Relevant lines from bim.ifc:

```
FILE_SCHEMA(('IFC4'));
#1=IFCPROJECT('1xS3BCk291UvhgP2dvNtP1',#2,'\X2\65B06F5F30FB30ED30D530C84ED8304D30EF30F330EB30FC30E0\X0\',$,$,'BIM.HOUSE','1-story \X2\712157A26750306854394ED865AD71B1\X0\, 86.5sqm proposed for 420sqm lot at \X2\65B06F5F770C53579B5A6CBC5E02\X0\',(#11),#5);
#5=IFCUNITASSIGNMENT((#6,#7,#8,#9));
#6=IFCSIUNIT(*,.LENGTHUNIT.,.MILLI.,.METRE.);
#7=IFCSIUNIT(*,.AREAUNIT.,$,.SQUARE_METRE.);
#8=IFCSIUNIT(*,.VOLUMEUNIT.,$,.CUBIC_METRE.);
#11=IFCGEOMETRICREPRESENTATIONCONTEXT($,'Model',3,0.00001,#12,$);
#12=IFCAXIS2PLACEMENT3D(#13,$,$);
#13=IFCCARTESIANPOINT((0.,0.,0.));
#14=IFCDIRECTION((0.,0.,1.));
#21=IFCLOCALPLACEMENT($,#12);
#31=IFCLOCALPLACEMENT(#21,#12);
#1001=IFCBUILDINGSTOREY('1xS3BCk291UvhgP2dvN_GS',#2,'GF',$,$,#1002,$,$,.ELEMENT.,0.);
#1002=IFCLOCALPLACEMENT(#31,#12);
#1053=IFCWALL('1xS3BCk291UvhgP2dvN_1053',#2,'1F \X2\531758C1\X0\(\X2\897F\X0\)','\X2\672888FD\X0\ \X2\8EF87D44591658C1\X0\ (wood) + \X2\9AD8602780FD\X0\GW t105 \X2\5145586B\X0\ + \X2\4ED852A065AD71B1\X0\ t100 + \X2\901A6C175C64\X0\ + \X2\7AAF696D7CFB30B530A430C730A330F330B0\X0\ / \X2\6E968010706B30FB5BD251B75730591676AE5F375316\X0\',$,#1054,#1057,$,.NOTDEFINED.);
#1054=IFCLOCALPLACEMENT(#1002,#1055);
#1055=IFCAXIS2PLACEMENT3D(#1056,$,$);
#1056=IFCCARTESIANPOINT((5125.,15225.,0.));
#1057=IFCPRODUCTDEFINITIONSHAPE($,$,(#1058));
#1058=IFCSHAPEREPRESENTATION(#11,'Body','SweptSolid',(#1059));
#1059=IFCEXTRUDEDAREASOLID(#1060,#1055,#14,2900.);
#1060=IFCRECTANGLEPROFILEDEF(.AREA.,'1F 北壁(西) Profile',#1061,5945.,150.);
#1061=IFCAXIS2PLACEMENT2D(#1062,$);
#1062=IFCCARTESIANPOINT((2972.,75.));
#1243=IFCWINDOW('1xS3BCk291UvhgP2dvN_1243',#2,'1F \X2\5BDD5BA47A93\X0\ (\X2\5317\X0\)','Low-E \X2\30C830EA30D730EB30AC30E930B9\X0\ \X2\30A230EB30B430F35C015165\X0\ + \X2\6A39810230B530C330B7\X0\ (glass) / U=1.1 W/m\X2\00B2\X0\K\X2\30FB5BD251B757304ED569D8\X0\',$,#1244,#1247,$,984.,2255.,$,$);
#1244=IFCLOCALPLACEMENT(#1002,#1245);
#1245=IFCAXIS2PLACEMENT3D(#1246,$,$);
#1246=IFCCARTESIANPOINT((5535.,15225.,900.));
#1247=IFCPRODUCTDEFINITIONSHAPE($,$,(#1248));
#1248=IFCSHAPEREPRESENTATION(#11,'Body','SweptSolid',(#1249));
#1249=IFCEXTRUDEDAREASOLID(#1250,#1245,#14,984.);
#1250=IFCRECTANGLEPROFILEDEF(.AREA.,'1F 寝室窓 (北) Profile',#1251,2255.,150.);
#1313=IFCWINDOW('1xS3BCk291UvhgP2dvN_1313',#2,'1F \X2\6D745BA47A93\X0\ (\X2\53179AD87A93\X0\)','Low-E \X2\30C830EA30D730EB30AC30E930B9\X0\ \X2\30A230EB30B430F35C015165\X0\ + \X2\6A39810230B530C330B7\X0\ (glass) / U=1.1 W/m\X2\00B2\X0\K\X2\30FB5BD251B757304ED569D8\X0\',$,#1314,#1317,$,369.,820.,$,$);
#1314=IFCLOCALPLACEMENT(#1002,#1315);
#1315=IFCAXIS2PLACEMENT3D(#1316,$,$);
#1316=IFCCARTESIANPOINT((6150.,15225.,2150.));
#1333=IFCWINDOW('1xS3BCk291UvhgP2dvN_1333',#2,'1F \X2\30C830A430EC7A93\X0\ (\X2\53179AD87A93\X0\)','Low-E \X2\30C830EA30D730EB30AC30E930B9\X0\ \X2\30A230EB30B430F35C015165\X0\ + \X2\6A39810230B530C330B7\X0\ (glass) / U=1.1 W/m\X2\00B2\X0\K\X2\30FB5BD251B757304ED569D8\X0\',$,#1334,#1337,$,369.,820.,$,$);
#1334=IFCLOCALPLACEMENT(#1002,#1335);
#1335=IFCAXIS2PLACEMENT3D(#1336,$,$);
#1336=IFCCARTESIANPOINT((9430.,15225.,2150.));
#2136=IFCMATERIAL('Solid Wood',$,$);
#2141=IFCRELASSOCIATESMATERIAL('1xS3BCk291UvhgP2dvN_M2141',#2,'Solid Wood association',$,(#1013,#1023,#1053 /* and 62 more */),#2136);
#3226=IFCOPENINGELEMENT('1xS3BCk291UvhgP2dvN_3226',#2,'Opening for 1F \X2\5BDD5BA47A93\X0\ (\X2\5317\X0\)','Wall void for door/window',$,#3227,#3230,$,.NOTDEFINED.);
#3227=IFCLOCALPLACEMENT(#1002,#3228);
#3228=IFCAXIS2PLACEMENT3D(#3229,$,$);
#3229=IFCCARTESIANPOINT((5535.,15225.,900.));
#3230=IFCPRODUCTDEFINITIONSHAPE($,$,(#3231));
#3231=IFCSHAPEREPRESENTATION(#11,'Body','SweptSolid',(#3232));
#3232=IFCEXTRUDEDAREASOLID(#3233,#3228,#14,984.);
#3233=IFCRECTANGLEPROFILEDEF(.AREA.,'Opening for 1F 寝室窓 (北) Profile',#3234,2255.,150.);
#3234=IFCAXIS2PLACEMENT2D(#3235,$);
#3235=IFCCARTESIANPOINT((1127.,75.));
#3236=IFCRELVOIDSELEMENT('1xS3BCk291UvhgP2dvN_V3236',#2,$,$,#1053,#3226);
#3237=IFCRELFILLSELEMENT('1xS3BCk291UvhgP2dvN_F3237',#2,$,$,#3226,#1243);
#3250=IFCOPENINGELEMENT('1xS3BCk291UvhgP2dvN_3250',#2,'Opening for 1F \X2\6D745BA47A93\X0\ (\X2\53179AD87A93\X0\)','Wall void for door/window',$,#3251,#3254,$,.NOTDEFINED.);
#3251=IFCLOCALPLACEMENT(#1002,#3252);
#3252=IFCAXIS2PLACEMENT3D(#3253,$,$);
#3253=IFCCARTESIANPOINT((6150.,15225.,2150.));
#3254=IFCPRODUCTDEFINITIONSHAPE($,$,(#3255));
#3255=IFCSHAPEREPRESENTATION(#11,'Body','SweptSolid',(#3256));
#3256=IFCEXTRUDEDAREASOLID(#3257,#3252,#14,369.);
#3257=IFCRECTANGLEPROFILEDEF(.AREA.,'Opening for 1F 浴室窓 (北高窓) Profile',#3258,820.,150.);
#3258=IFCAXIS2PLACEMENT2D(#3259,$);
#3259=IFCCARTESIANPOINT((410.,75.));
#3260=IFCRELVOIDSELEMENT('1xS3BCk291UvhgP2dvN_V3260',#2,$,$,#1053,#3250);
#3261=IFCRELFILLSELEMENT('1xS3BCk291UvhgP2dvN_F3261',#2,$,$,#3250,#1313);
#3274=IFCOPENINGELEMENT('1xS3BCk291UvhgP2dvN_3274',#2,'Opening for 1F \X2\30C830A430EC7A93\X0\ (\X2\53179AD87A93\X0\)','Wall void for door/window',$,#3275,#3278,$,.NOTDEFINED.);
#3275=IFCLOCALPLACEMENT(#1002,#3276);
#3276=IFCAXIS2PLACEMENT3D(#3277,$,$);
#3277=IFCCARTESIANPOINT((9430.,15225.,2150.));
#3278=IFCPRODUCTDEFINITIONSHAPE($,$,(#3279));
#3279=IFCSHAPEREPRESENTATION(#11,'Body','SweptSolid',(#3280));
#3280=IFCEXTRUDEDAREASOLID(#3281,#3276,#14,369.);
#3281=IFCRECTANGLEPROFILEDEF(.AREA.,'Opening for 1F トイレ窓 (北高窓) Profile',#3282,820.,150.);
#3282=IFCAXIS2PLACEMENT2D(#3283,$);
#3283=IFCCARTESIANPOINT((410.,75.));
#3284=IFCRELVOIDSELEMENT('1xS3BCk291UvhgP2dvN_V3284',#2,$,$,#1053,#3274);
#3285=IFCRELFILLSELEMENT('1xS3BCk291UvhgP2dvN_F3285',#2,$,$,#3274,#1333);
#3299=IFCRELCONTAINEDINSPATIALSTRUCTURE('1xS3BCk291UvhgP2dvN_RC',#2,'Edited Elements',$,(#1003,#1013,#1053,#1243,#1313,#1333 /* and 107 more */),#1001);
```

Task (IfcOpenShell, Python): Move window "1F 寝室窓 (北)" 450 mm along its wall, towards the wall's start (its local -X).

```python
import ifcopenshell
import ifcopenshell.api.geometry
import ifcopenshell.util.placement
import ifcopenshell.util.unit

model = ifcopenshell.open("bim.ifc")
unit_scale = ifcopenshell.util.unit.calculate_unit_scale(model)

window = model.by_id(1243)
opening = window.FillsVoids[0].RelatingOpeningElement
wall = opening.VoidsElements[0].RelatingBuildingElement

wall_matrix = ifcopenshell.util.placement.get_local_placement(wall.ObjectPlacement)
shift = wall_matrix[:3, 0] * -0.45 / unit_scale
before = ifcopenshell.util.placement.get_local_placement(window.ObjectPlacement)[:3, 3].copy()

# The window is not placed relative to its opening, so move both.
for product in (opening, window):
    matrix = ifcopenshell.util.placement.get_local_placement(product.ObjectPlacement)
    matrix[:3, 3] += shift
    ifcopenshell.api.geometry.edit_object_placement(model, product=product, matrix=matrix, is_si=False)

after = ifcopenshell.util.placement.get_local_placement(window.ObjectPlacement)[:3, 3]
print("window moved by", (after - before).round(3) + 0.0)

model.write("bim_rev.ifc")
```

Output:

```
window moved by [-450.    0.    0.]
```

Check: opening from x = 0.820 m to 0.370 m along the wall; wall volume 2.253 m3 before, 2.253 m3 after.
